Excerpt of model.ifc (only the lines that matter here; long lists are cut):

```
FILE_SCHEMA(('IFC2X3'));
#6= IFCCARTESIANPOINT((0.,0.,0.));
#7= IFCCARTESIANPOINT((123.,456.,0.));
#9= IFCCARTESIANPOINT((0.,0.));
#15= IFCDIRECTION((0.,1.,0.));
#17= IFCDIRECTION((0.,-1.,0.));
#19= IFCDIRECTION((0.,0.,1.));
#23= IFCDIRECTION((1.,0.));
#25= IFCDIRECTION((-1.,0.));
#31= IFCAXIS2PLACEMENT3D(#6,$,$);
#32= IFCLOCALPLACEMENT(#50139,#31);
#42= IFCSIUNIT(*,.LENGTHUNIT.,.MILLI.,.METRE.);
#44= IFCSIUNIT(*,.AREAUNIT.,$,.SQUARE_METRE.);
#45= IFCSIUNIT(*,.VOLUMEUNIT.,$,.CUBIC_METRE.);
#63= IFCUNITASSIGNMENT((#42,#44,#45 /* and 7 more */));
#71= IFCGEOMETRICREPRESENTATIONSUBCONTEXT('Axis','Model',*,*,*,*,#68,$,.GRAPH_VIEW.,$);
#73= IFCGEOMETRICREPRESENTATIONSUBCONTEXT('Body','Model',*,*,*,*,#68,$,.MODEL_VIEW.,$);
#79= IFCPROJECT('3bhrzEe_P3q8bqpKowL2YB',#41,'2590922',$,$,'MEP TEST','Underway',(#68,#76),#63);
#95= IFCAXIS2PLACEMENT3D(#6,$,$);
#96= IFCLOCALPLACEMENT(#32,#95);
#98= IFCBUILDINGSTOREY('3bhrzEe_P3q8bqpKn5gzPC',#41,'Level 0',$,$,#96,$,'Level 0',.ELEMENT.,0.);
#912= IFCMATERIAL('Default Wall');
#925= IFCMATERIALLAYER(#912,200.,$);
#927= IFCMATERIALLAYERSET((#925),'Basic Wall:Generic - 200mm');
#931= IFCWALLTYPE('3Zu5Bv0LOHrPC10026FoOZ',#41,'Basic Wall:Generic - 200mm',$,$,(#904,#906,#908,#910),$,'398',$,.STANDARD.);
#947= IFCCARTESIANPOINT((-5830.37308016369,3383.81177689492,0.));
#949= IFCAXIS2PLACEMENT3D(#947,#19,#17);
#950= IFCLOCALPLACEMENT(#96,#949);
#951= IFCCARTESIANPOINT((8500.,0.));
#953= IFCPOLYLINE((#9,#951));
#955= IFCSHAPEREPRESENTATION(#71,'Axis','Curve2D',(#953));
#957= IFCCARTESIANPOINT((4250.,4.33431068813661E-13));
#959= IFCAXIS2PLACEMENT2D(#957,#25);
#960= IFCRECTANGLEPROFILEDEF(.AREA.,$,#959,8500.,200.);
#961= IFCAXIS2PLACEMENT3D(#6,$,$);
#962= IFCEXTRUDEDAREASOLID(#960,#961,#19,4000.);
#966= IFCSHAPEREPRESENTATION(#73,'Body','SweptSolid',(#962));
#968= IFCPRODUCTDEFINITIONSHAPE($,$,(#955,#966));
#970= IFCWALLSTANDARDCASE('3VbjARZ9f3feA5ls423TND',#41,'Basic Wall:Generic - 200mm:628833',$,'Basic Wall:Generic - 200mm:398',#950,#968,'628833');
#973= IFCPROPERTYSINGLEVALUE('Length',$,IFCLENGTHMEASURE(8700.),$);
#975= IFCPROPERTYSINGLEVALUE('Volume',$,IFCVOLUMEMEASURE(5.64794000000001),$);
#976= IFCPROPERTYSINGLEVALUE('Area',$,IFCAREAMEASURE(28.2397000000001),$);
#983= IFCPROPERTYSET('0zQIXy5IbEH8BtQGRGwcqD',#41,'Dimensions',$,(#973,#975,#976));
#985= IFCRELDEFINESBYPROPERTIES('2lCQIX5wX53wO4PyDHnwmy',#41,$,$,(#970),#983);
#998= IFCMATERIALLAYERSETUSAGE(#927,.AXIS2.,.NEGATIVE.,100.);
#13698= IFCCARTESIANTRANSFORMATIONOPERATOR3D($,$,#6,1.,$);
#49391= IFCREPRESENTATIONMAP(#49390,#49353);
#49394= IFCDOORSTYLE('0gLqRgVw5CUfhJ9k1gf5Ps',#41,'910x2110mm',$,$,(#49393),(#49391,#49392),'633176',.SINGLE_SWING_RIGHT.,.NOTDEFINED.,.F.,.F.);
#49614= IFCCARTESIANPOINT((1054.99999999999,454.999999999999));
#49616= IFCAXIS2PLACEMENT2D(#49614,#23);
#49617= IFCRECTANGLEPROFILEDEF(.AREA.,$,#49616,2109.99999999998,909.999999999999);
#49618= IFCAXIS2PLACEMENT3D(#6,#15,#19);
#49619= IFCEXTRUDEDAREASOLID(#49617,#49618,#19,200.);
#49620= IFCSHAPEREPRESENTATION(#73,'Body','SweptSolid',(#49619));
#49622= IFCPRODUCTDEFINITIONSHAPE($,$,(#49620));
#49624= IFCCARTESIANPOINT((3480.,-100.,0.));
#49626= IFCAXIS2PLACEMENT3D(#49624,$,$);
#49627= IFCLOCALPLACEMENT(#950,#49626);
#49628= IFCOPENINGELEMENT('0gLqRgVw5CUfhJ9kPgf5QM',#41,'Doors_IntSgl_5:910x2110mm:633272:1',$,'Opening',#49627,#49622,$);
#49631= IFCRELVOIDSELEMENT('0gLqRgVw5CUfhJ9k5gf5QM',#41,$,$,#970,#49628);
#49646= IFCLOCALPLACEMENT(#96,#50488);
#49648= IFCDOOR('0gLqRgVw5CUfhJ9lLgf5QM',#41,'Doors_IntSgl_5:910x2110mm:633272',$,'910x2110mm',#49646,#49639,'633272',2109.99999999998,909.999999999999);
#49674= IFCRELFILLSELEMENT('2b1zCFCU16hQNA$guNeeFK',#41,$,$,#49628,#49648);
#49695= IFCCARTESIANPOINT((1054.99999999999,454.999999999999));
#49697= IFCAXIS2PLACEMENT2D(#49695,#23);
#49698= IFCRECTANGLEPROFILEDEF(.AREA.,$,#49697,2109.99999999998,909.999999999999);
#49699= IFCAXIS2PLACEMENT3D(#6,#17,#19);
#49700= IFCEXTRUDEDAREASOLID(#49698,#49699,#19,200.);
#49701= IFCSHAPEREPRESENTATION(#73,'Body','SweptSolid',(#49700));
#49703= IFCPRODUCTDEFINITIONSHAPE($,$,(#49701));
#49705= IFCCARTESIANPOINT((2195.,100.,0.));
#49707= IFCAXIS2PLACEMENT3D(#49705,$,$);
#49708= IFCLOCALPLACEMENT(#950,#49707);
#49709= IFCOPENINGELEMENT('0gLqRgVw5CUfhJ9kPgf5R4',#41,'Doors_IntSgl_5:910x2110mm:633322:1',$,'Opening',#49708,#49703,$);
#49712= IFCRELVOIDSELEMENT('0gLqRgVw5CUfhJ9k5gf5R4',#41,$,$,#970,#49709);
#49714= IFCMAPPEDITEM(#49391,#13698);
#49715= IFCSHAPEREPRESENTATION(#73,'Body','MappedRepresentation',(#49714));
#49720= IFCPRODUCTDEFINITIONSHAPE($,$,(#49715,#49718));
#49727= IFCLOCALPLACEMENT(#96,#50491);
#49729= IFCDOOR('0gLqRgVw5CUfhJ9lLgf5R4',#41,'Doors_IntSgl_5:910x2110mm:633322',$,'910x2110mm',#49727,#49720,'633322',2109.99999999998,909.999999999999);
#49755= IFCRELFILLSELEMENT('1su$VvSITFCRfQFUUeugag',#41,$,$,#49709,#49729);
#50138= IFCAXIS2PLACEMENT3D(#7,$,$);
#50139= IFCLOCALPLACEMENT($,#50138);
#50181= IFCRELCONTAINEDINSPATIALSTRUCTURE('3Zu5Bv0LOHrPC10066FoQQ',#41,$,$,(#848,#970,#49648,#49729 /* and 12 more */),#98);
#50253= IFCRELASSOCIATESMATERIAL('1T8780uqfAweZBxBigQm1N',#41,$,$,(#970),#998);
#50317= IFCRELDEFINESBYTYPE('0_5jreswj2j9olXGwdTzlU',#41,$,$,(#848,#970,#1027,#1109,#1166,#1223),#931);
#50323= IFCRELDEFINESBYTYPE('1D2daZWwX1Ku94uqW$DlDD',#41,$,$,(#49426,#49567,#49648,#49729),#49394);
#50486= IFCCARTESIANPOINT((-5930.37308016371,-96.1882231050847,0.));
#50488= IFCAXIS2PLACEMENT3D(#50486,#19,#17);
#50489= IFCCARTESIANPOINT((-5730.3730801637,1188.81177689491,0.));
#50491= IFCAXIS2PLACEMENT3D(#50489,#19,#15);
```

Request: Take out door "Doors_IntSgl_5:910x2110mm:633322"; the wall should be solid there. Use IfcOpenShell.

```python
import ifcopenshell
import ifcopenshell.api.feature
import ifcopenshell.api.pset
import ifcopenshell.api.root
import ifcopenshell.geom
import ifcopenshell.util.element
import ifcopenshell.util.shape
import ifcopenshell.util.unit

model = ifcopenshell.open("model.ifc")
area_scale = ifcopenshell.util.unit.calculate_unit_scale(model, "AREAUNIT")
volume_scale = ifcopenshell.util.unit.calculate_unit_scale(model, "VOLUMEUNIT")
settings = ifcopenshell.geom.settings()


def volume(element):
    """Net volume in cubic metres, openings subtracted."""
    shape = ifcopenshell.geom.create_shape(settings, element)
    return ifcopenshell.util.shape.get_volume(shape.geometry)


door = model.by_id(49729)
opening = door.FillsVoids[0].RelatingOpeningElement
wall = opening.VoidsElements[0].RelatingBuildingElement
before = volume(wall)

ifcopenshell.api.root.remove_product(model, product=door)
ifcopenshell.api.feature.remove_feature(model, feature=opening)

after = volume(wall)
thickness = 0.2  # wall thickness in metres

# Update the wall's stored quantities.
pset = model.by_id(ifcopenshell.util.element.get_pset(wall, "Dimensions", should_inherit=False)["id"])
ifcopenshell.api.pset.edit_pset(model, pset=pset, properties={
    "Volume": model.create_entity("IfcVolumeMeasure", after / volume_scale),
    "Area": model.create_entity("IfcAreaMeasure", after / thickness / area_scale),
})

print(f"wall volume {before:.3f} -> {after:.3f} m3")

model.write("model_edited.ifc")
```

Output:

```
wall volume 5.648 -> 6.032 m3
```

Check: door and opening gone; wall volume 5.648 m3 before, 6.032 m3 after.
